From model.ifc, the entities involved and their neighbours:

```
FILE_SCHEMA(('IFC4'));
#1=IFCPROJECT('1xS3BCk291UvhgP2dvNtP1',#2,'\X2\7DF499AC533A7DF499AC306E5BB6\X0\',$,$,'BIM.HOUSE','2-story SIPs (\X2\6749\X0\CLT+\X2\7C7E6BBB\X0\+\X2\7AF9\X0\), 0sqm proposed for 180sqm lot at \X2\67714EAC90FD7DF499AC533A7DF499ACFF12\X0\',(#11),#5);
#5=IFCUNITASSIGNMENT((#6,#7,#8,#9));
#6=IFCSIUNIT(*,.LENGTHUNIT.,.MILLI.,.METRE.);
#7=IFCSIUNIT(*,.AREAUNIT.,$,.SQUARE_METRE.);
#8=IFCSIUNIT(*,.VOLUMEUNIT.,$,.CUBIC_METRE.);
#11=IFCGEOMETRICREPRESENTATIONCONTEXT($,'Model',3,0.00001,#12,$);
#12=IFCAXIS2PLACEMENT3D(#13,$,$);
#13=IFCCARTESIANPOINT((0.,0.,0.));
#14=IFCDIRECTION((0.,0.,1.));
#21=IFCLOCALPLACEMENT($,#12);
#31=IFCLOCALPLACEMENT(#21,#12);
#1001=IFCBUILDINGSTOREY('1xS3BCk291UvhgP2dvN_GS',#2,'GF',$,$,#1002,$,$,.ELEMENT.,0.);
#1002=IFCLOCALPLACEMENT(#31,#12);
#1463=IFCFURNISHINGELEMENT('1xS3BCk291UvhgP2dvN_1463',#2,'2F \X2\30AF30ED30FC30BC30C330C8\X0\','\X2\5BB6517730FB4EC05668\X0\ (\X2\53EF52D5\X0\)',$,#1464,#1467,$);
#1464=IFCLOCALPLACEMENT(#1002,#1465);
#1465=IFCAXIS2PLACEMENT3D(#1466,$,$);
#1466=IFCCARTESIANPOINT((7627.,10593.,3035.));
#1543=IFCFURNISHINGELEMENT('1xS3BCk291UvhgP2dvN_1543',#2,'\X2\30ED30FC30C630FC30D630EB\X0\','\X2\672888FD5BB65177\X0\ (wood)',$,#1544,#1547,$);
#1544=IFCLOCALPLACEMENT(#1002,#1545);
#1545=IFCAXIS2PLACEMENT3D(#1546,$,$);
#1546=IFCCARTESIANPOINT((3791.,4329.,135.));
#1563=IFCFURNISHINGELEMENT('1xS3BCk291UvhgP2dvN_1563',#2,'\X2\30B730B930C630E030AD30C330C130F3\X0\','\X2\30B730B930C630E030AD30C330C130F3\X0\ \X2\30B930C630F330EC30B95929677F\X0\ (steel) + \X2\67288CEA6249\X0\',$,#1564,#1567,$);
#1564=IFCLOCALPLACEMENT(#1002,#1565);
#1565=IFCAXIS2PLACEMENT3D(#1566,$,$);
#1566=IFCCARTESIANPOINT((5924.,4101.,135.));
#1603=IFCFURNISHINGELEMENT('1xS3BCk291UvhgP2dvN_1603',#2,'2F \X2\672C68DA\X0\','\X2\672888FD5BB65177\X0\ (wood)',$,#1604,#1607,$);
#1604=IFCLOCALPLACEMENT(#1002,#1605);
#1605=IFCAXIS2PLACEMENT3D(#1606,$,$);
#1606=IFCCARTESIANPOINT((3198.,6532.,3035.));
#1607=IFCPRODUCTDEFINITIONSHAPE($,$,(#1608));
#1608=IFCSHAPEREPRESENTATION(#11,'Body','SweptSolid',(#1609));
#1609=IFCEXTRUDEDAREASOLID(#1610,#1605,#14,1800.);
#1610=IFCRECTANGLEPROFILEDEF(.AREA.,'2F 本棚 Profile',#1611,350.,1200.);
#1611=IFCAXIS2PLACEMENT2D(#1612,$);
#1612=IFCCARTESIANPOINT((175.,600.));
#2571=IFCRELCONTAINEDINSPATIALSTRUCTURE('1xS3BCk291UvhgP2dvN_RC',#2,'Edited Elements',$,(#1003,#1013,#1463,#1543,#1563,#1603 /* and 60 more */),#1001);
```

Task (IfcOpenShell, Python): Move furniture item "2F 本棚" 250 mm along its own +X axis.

```python
import ifcopenshell
import ifcopenshell.api.geometry
import ifcopenshell.util.placement
import ifcopenshell.util.unit

model = ifcopenshell.open("model.ifc")
unit_scale = ifcopenshell.util.unit.calculate_unit_scale(model)

item = model.by_id(1603)
matrix = ifcopenshell.util.placement.get_local_placement(item.ObjectPlacement)
matrix[:3, 3] += matrix[:3, 0] * 0.25 / unit_scale
ifcopenshell.api.geometry.edit_object_placement(model, product=item, matrix=matrix, is_si=False)

print(ifcopenshell.util.placement.get_local_placement(item.ObjectPlacement).round(3) + 0.0)

model.write("model_v2.ifc")
```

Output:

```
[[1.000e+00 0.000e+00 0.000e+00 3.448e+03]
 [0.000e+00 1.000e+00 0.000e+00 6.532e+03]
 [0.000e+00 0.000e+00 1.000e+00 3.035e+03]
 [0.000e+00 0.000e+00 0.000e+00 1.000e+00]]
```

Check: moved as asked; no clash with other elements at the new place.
